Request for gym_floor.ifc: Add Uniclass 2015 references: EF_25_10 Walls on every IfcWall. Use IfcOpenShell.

First a look at what the model holds.

```python
import ifcopenshell

model = ifcopenshell.open("gym_floor.ifc")
print(model.schema)
print("classifications:", [c.Name for c in model.by_type("IfcClassification")])
for ifc_class in ("IfcDoor", "IfcRoof", "IfcStair", "IfcWall", "IfcWindow"):
    print(ifc_class, len(model.by_type(ifc_class)))
```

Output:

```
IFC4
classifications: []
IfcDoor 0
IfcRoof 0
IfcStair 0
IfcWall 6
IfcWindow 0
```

```python
import ifcopenshell
import ifcopenshell.api.classification

model = ifcopenshell.open("gym_floor.ifc")

system = ifcopenshell.api.classification.add_classification(model, classification="Uniclass 2015")

codes = {
    "IfcWall": ("EF_25_10", "Walls"),
}
for ifc_class, (code, name) in codes.items():
    products = model.by_type(ifc_class)
    ifcopenshell.api.classification.add_reference(
        model, products=products, classification=system, identification=code, name=name
    )
    print(code, len(products))

model.write("gym_floor_updated.ifc")
```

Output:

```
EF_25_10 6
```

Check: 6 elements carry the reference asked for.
